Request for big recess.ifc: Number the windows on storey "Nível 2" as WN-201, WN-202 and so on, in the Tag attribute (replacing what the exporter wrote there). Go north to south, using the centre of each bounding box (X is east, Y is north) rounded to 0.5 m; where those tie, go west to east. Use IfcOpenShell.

First a look at what the model holds.

```python
import ifcopenshell
import ifcopenshell.util.element
import ifcopenshell.util.placement

model = ifcopenshell.open("big recess.ifc")
print(model.schema)
storey = next(s for s in model.by_type("IfcBuildingStorey") if s.Name == "Nível 2")
windows = [e for e in ifcopenshell.util.element.get_decomposition(storey) if e.is_a("IfcWindow")]
for e in sorted(windows, key=lambda e: e.id()):
    origin = ifcopenshell.util.placement.get_local_placement(e.ObjectPlacement)[:3, 3]
    print(e.id(), e.Tag, e.Name, origin.round(2) + 0.0, sep=" | ")
```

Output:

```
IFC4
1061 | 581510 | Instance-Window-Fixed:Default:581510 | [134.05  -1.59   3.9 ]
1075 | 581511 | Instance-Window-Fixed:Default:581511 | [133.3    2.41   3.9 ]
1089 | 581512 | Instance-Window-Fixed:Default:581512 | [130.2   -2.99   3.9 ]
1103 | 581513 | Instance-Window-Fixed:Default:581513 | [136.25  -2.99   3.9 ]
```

```python
import ifcopenshell
import ifcopenshell.geom
import ifcopenshell.util.element
import ifcopenshell.util.shape

model = ifcopenshell.open("big recess.ifc")
settings = ifcopenshell.geom.settings()
settings.set("use-world-coords", True)


def centre(element):
    shape = ifcopenshell.geom.create_shape(settings, element)
    return ifcopenshell.util.shape.get_bbox_centroid(shape.geometry)


storey = next(s for s in model.by_type("IfcBuildingStorey") if s.Name == "Nível 2")
windows = [e for e in ifcopenshell.util.element.get_decomposition(storey) if e.is_a("IfcWindow")]

# Insertion points can sit at a corner or the storey origin, so sort by the geometry (in metres).
centres = {e: centre(e) for e in windows}
windows.sort(key=lambda e: (-round(centres[e][1] / 0.5), centres[e][0]))

for i, e in enumerate(windows, start=1):
    number = f"WN-2{i:02d}"
    e.Tag = number
    print(e.id(), number)

model.write("big recess_updated.ifc")
```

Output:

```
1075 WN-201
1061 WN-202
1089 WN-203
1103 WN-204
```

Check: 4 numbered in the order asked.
